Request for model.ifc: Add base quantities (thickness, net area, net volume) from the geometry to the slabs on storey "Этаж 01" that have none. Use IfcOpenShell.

First a look at what the model holds.

```python
import ifcopenshell
import ifcopenshell.util.element
import ifcopenshell.util.unit

model = ifcopenshell.open("model.ifc")
print(model.schema)
for unit_type in ("LENGTHUNIT", "AREAUNIT", "VOLUMEUNIT"):
    print(unit_type, ifcopenshell.util.unit.calculate_unit_scale(model, unit_type))
storey = next(s for s in model.by_type("IfcBuildingStorey") if s.Name == "Этаж 01")
slabs = [e for e in ifcopenshell.util.element.get_decomposition(storey) if e.is_a("IfcSlab")]
for e in sorted(slabs, key=lambda e: e.id()):
    print(e.id(), e.is_a(), e.Name, list(ifcopenshell.util.element.get_psets(e, qtos_only=True)), sep=" | ")
```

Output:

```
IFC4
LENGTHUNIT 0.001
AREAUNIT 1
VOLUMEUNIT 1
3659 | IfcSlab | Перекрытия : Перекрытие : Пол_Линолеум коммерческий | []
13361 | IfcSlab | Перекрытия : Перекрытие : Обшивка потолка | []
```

```python
import ifcopenshell
import ifcopenshell.api.pset
import ifcopenshell.geom
import ifcopenshell.util.element
import ifcopenshell.util.shape
import ifcopenshell.util.unit

model = ifcopenshell.open("model.ifc")
unit_scale = ifcopenshell.util.unit.calculate_unit_scale(model)
area_scale = ifcopenshell.util.unit.calculate_unit_scale(model, "AREAUNIT")
volume_scale = ifcopenshell.util.unit.calculate_unit_scale(model, "VOLUMEUNIT")
settings = ifcopenshell.geom.settings()

storey = next(s for s in model.by_type("IfcBuildingStorey") if s.Name == "Этаж 01")
slabs = [e for e in ifcopenshell.util.element.get_decomposition(storey) if e.is_a("IfcSlab")]

for e in sorted(slabs, key=lambda e: e.id()):
    if ifcopenshell.util.element.get_psets(e, qtos_only=True, should_inherit=False):
        continue
    # Geometry comes back in metres, in the element's own axes.
    shape = ifcopenshell.geom.create_shape(settings, e)
    values = {
        "Width": ifcopenshell.util.shape.get_z(shape.geometry) / unit_scale,
        "NetArea": ifcopenshell.util.shape.get_footprint_area(shape.geometry) / area_scale,
        "NetVolume": ifcopenshell.util.shape.get_volume(shape.geometry) / volume_scale,
    }
    qto = ifcopenshell.api.pset.add_qto(model, product=e, name="Qto_SlabBaseQuantities")
    ifcopenshell.api.pset.edit_qto(model, qto=qto, properties=values)
    print(e.id(), {k: round(v, 3) for k, v in values.items()})

model.write("model_updated.ifc")
```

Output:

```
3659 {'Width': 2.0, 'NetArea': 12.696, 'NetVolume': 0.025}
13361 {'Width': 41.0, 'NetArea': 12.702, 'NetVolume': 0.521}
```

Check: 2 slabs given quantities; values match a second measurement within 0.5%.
